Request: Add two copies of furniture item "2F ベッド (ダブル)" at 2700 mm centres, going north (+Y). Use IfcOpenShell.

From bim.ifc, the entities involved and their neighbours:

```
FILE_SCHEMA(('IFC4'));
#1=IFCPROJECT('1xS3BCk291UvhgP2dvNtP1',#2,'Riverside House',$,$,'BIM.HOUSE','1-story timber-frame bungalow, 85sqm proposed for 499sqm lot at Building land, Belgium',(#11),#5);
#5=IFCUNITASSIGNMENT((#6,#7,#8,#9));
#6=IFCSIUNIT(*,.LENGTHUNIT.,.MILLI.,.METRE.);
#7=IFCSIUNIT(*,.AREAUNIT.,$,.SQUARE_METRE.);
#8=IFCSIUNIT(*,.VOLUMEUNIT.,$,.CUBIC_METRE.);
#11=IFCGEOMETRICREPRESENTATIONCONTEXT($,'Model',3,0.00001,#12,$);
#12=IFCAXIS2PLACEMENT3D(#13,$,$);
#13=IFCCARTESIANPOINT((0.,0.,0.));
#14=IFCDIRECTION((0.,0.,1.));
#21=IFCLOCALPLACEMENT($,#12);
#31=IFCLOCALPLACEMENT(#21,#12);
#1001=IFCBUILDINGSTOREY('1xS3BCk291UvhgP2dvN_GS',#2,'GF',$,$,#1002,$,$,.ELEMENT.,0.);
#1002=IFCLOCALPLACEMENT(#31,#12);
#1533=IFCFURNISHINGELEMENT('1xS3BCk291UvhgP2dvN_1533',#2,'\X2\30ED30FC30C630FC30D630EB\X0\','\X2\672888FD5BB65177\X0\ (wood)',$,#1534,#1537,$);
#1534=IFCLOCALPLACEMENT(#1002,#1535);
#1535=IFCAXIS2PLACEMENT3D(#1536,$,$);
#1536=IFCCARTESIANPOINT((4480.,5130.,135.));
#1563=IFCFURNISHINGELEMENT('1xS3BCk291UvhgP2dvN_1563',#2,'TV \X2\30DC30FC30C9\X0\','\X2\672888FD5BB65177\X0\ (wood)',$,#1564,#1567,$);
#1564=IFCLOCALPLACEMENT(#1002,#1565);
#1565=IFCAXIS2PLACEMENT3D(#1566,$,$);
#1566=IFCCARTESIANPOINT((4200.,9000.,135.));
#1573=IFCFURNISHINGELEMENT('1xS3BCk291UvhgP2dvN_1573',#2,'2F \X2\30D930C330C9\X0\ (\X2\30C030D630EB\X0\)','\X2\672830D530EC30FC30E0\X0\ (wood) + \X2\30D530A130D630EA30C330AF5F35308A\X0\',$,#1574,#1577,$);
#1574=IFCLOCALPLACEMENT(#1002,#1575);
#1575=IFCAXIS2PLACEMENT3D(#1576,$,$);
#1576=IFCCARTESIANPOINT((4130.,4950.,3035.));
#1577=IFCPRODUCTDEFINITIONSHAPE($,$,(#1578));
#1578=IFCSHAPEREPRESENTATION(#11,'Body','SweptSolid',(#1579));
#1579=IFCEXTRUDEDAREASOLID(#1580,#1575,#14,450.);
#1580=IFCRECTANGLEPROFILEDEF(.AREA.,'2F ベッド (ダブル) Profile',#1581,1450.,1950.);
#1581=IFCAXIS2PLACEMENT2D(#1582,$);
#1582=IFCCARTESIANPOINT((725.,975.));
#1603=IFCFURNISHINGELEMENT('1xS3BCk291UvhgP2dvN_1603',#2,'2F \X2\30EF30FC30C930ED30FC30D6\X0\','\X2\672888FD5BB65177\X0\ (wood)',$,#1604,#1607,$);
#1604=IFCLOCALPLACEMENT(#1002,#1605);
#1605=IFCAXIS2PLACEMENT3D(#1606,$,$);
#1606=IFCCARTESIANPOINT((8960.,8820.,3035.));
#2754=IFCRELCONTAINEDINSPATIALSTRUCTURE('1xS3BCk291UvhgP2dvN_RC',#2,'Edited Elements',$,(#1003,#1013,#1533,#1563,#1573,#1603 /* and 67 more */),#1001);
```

```python
import numpy as np
import ifcopenshell
import ifcopenshell.api.geometry
import ifcopenshell.api.root
import ifcopenshell.util.element
import ifcopenshell.util.placement
import ifcopenshell.util.unit

model = ifcopenshell.open("bim.ifc")
unit_scale = ifcopenshell.util.unit.calculate_unit_scale(model)


def reuse_history(source, copy):
    """copy_class also copies each property set's owner history, people and application; keep the originals."""
    for rel in copy.IsDefinedBy:
        if rel.is_a("IfcRelDefinesByProperties") and (history := rel.RelatingPropertyDefinition.OwnerHistory):
            rel.RelatingPropertyDefinition.OwnerHistory = source.OwnerHistory
            ifcopenshell.util.element.remove_deep2(model, history)


source = model.by_guid("1xS3BCk291UvhgP2dvN_1573")
base = ifcopenshell.util.placement.get_local_placement(source.ObjectPlacement)
step = np.array([0.0, 1.0, 0.0]) * 2.7 / unit_scale

for i in range(1, 3):
    copy = ifcopenshell.api.root.copy_class(model, product=source)
    copy.Representation = ifcopenshell.util.element.copy_deep(
        model, source.Representation, exclude=["IfcGeometricRepresentationContext", "IfcRepresentationMap"]
    )
    reuse_history(source, copy)
    matrix = base.copy()
    matrix[:3, 3] += i * step
    print("added at", matrix[:3, 3].round(3) + 0.0)
    ifcopenshell.api.geometry.edit_object_placement(model, product=copy, matrix=matrix, is_si=False)

model.write("bim_rev.ifc")
```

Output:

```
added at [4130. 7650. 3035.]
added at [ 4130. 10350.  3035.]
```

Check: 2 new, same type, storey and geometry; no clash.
